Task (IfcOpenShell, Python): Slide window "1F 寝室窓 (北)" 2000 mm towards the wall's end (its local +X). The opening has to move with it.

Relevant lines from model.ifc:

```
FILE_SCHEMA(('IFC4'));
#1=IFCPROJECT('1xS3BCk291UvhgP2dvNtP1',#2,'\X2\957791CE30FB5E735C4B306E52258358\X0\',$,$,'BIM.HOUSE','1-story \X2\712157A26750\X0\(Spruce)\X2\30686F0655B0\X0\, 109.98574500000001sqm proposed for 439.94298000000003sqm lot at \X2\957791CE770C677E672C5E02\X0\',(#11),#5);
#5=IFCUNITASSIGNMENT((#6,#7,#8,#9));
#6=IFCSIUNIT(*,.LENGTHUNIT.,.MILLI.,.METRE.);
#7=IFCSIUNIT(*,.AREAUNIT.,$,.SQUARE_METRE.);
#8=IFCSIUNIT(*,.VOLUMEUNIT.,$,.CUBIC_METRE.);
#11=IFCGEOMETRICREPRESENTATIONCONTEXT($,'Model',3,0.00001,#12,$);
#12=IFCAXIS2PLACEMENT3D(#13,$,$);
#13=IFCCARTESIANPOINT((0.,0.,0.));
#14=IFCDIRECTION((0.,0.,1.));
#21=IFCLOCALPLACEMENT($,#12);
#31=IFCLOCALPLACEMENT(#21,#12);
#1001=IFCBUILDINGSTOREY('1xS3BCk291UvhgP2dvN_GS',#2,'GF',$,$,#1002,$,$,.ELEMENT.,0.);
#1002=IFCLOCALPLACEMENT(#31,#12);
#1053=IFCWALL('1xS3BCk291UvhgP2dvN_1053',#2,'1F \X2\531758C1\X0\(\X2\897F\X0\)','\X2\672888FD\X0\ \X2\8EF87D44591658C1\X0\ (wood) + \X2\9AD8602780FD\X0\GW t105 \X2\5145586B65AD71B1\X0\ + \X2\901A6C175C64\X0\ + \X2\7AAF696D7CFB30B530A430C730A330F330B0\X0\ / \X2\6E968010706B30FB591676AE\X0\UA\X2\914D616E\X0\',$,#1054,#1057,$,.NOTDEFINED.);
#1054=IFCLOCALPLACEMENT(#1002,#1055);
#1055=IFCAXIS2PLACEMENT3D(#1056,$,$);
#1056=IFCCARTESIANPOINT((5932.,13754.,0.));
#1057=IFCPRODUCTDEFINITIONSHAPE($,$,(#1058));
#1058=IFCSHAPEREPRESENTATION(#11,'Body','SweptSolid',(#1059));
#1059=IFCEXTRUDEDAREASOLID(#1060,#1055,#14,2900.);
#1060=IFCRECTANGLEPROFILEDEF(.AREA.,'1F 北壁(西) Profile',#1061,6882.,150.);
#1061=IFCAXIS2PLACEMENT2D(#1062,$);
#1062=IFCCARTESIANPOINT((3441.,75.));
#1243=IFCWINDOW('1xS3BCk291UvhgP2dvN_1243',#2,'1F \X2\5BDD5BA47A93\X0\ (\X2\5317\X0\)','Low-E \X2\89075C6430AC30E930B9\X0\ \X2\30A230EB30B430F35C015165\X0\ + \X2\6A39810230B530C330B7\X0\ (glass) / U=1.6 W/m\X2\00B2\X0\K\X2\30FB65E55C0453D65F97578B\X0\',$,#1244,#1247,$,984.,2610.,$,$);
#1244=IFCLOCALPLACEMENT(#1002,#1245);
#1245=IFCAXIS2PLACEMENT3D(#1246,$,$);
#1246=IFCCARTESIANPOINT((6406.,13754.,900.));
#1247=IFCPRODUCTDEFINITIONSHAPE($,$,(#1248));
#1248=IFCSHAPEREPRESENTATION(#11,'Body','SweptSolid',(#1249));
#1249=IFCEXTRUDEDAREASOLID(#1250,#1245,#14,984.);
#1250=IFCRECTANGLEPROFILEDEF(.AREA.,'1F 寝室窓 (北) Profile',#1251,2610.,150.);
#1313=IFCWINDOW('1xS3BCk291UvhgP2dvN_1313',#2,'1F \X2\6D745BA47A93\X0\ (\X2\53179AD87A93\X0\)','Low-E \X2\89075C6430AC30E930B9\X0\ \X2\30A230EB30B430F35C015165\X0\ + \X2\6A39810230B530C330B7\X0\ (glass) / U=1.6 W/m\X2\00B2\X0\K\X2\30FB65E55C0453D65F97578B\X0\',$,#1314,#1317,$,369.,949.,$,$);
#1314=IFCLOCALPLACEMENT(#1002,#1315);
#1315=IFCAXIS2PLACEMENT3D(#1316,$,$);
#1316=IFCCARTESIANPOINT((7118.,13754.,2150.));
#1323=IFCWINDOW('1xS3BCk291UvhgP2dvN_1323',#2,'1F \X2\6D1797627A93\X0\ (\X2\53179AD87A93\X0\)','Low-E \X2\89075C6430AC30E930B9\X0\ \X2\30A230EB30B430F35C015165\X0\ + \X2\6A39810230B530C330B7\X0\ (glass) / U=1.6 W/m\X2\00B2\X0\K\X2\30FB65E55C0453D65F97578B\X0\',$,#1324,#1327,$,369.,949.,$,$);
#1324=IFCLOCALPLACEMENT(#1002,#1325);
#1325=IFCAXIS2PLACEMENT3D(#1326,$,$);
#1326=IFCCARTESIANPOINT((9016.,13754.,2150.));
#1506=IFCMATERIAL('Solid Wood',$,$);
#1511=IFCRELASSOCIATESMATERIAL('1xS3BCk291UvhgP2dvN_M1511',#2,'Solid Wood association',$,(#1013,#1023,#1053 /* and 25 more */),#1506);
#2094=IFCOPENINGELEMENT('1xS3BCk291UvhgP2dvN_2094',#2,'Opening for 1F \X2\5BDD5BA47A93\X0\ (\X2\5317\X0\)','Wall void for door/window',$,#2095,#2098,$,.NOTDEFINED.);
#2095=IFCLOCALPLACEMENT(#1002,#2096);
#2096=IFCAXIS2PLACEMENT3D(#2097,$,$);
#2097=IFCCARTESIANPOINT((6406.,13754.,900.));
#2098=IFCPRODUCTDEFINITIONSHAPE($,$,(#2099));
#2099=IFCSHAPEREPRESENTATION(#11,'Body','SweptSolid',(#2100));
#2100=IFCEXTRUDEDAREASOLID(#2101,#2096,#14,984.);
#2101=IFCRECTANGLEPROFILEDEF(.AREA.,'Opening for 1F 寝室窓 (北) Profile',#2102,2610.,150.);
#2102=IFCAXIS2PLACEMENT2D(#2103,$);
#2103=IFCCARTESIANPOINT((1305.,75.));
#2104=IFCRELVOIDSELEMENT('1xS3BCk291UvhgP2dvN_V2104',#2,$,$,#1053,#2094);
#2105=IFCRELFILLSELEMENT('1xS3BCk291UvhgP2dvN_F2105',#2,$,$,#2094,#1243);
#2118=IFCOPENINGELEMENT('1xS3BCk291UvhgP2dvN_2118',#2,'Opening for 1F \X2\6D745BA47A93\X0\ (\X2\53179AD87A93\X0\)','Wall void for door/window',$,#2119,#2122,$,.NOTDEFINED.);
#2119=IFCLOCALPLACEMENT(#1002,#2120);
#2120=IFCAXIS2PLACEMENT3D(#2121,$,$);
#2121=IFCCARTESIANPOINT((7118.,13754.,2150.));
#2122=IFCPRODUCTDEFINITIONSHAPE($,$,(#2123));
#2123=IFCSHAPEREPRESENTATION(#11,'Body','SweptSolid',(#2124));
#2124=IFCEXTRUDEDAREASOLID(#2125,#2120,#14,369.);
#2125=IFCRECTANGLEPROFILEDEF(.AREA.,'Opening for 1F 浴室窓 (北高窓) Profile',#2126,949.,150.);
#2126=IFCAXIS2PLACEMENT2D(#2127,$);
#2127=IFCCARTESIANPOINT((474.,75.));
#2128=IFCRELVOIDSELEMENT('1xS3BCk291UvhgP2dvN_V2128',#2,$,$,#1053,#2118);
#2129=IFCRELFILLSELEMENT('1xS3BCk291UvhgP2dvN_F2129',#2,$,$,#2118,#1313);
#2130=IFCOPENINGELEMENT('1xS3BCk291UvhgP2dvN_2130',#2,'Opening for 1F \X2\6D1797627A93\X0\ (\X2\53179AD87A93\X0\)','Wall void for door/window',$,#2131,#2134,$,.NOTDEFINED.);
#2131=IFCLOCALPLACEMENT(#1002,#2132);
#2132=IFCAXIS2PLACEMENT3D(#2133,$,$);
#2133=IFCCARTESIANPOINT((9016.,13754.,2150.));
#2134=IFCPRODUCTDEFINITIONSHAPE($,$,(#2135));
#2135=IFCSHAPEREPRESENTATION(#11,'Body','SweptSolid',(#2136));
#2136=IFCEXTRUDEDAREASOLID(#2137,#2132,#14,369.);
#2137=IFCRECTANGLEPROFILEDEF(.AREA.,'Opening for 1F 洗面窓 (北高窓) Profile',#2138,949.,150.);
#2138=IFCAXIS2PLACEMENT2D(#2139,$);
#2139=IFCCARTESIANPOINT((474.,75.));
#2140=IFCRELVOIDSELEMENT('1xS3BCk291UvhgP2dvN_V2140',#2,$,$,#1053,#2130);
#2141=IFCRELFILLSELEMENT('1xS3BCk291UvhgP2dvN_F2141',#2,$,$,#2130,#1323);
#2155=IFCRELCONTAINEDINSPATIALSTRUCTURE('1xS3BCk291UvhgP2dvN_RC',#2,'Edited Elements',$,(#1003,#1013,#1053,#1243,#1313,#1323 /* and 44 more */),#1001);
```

```python
import ifcopenshell
import ifcopenshell.api.geometry
import ifcopenshell.util.placement

model = ifcopenshell.open("model.ifc")

window = model.by_id(1243)
opening = window.FillsVoids[0].RelatingOpeningElement
wall = opening.VoidsElements[0].RelatingBuildingElement

wall_matrix = ifcopenshell.util.placement.get_local_placement(wall.ObjectPlacement)
shift = wall_matrix[:3, 0] * 2000.0
before = ifcopenshell.util.placement.get_local_placement(window.ObjectPlacement)[:3, 3].copy()

# The window is not placed relative to its opening, so move both.
for product in (opening, window):
    matrix = ifcopenshell.util.placement.get_local_placement(product.ObjectPlacement)
    matrix[:3, 3] += shift
    ifcopenshell.api.geometry.edit_object_placement(model, product=product, matrix=matrix, is_si=False)

after = ifcopenshell.util.placement.get_local_placement(window.ObjectPlacement)[:3, 3]
print("window moved by", (after - before).round(3) + 0.0)

model.write("model_v2.ifc")
```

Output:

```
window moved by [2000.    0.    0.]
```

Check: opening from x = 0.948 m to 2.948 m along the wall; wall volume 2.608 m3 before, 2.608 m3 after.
